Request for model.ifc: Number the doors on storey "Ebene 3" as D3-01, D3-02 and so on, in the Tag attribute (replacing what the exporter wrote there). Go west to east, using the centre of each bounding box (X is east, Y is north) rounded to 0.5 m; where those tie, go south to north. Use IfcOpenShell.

First a look at what the model holds.

```python
import ifcopenshell
import ifcopenshell.util.element
import ifcopenshell.util.placement

model = ifcopenshell.open("model.ifc")
print(model.schema)
storey = next(s for s in model.by_type("IfcBuildingStorey") if s.Name == "Ebene 3")
doors = [e for e in ifcopenshell.util.element.get_decomposition(storey) if e.is_a("IfcDoor")]
for e in sorted(doors, key=lambda e: e.id()):
    origin = ifcopenshell.util.placement.get_local_placement(e.ObjectPlacement)[:3, 3]
    print(e.id(), e.Tag, e.Name, origin.round(2) + 0.0, sep=" | ")
```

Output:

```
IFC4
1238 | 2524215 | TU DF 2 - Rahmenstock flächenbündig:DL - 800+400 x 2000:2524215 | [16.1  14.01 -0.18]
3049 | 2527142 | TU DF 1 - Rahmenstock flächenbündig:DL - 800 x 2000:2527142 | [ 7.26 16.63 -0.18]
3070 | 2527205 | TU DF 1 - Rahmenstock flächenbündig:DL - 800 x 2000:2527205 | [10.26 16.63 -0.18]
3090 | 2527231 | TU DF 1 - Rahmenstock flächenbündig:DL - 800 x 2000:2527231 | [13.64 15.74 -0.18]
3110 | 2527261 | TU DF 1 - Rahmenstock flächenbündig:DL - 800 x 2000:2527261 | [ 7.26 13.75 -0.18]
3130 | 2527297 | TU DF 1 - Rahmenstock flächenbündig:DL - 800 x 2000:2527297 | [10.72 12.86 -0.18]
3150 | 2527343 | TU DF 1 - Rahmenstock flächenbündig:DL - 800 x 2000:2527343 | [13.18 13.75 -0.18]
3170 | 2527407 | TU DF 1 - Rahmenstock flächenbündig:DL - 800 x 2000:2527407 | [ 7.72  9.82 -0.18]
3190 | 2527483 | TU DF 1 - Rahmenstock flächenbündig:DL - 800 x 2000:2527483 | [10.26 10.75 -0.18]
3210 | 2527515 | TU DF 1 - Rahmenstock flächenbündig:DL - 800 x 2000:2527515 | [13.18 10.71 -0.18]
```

```python
import ifcopenshell
import ifcopenshell.geom
import ifcopenshell.util.element
import ifcopenshell.util.shape

model = ifcopenshell.open("model.ifc")
settings = ifcopenshell.geom.settings()
settings.set("use-world-coords", True)


def centre(element):
    shape = ifcopenshell.geom.create_shape(settings, element)
    return ifcopenshell.util.shape.get_bbox_centroid(shape.geometry)


storey = next(s for s in model.by_type("IfcBuildingStorey") if s.Name == "Ebene 3")
doors = [e for e in ifcopenshell.util.element.get_decomposition(storey) if e.is_a("IfcDoor")]

# Insertion points can sit at a corner or the storey origin, so sort by the geometry (in metres).
centres = {e: centre(e) for e in doors}
doors.sort(key=lambda e: (round(centres[e][0] / 0.5), centres[e][1]))

for i, e in enumerate(doors, start=1):
    number = f"D3-{i:02d}"
    e.Tag = number
    print(e.id(), number)

model.write("model-out.ifc")
```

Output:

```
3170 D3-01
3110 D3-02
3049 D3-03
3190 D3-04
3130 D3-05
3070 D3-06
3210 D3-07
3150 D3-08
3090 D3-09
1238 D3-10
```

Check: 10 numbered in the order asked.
